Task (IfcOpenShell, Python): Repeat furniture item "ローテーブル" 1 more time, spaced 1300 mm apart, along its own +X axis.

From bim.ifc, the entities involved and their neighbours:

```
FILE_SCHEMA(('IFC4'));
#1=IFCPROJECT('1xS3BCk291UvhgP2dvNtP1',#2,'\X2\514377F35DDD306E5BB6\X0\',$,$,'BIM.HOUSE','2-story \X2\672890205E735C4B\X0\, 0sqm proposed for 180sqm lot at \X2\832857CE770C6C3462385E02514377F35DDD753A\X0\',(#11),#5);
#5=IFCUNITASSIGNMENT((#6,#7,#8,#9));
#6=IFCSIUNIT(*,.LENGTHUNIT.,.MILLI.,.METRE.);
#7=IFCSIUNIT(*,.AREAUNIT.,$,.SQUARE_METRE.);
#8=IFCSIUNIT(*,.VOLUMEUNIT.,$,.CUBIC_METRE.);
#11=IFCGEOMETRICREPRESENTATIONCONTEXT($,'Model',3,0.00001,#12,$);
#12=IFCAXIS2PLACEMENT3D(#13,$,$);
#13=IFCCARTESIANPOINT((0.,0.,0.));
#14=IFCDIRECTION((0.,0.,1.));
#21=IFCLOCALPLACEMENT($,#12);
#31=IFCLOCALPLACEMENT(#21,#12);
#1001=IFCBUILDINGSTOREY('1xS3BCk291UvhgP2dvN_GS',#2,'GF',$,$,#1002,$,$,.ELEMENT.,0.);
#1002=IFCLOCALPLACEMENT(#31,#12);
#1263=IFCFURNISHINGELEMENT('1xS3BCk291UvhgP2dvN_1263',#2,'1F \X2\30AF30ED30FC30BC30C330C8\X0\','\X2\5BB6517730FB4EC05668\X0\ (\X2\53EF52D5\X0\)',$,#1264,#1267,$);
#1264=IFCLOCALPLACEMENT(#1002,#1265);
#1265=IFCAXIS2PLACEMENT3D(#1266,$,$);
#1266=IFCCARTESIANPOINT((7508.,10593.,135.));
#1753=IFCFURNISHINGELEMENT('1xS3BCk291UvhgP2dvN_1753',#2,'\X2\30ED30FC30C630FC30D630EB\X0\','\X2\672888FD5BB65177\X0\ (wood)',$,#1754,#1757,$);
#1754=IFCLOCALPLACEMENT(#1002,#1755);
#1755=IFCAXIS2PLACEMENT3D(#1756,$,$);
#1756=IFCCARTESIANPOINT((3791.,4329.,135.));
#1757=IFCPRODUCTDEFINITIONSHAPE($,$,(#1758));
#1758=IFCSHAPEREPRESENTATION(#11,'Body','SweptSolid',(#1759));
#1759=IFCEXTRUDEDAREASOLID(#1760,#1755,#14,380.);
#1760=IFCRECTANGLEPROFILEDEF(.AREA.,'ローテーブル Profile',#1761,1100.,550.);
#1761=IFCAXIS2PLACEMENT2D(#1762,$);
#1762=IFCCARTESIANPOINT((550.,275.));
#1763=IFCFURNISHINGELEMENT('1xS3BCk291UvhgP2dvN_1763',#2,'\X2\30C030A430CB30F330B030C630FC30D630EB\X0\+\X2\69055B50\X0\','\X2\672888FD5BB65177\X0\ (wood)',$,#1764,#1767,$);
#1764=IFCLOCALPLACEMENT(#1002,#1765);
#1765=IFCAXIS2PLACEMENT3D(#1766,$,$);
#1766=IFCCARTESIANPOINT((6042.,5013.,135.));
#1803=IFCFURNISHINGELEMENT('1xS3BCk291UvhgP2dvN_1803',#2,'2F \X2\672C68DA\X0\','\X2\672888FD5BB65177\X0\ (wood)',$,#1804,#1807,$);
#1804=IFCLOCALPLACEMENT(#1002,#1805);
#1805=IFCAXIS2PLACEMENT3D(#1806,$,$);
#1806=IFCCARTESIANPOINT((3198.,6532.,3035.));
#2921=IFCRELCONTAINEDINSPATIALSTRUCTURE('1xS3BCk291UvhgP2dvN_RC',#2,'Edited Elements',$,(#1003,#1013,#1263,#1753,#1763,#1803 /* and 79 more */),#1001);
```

```python
import ifcopenshell
import ifcopenshell.api.geometry
import ifcopenshell.api.root
import ifcopenshell.util.element
import ifcopenshell.util.placement

model = ifcopenshell.open("bim.ifc")


def reuse_history(source, copy):
    """copy_class also copies each property set's owner history, people and application; keep the originals."""
    for rel in copy.IsDefinedBy:
        if rel.is_a("IfcRelDefinesByProperties") and (history := rel.RelatingPropertyDefinition.OwnerHistory):
            rel.RelatingPropertyDefinition.OwnerHistory = source.OwnerHistory
            ifcopenshell.util.element.remove_deep2(model, history)


source = model.by_guid("1xS3BCk291UvhgP2dvN_1753")
base = ifcopenshell.util.placement.get_local_placement(source.ObjectPlacement)
step = base[:3, 0] * 1300.0

for i in range(1, 2):
    copy = ifcopenshell.api.root.copy_class(model, product=source)
    copy.Representation = ifcopenshell.util.element.copy_deep(
        model, source.Representation, exclude=["IfcGeometricRepresentationContext", "IfcRepresentationMap"]
    )
    reuse_history(source, copy)
    matrix = base.copy()
    matrix[:3, 3] += i * step
    print("added at", matrix[:3, 3].round(3) + 0.0)
    ifcopenshell.api.geometry.edit_object_placement(model, product=copy, matrix=matrix, is_si=False)

model.write("bim_edited.ifc")
```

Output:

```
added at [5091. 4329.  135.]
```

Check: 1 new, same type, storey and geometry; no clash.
